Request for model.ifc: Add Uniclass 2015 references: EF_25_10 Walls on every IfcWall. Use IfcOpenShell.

First a look at what the model holds.

```python
import ifcopenshell

model = ifcopenshell.open("model.ifc")
print(model.schema)
print("classifications:", [c.Name for c in model.by_type("IfcClassification")])
for ifc_class in ("IfcDoor", "IfcRoof", "IfcStair", "IfcWall", "IfcWindow"):
    print(ifc_class, len(model.by_type(ifc_class)))
```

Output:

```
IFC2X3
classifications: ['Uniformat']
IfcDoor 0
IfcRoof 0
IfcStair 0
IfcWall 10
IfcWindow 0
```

```python
import ifcopenshell
import ifcopenshell.api.classification

model = ifcopenshell.open("model.ifc")

# IFC2X3 requires Source and Edition and has no link from the project to the system.
system = model.create_entity("IfcClassification", Source="NBS", Edition="2015", Name="Uniclass 2015")

codes = {
    "IfcWall": ("EF_25_10", "Walls"),
}
for ifc_class, (code, name) in codes.items():
    products = model.by_type(ifc_class)
    ifcopenshell.api.classification.add_reference(
        model, products=products, classification=system, identification=code, name=name
    )
    print(code, len(products))

model.write("model_rev.ifc")
```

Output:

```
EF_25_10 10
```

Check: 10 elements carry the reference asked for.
